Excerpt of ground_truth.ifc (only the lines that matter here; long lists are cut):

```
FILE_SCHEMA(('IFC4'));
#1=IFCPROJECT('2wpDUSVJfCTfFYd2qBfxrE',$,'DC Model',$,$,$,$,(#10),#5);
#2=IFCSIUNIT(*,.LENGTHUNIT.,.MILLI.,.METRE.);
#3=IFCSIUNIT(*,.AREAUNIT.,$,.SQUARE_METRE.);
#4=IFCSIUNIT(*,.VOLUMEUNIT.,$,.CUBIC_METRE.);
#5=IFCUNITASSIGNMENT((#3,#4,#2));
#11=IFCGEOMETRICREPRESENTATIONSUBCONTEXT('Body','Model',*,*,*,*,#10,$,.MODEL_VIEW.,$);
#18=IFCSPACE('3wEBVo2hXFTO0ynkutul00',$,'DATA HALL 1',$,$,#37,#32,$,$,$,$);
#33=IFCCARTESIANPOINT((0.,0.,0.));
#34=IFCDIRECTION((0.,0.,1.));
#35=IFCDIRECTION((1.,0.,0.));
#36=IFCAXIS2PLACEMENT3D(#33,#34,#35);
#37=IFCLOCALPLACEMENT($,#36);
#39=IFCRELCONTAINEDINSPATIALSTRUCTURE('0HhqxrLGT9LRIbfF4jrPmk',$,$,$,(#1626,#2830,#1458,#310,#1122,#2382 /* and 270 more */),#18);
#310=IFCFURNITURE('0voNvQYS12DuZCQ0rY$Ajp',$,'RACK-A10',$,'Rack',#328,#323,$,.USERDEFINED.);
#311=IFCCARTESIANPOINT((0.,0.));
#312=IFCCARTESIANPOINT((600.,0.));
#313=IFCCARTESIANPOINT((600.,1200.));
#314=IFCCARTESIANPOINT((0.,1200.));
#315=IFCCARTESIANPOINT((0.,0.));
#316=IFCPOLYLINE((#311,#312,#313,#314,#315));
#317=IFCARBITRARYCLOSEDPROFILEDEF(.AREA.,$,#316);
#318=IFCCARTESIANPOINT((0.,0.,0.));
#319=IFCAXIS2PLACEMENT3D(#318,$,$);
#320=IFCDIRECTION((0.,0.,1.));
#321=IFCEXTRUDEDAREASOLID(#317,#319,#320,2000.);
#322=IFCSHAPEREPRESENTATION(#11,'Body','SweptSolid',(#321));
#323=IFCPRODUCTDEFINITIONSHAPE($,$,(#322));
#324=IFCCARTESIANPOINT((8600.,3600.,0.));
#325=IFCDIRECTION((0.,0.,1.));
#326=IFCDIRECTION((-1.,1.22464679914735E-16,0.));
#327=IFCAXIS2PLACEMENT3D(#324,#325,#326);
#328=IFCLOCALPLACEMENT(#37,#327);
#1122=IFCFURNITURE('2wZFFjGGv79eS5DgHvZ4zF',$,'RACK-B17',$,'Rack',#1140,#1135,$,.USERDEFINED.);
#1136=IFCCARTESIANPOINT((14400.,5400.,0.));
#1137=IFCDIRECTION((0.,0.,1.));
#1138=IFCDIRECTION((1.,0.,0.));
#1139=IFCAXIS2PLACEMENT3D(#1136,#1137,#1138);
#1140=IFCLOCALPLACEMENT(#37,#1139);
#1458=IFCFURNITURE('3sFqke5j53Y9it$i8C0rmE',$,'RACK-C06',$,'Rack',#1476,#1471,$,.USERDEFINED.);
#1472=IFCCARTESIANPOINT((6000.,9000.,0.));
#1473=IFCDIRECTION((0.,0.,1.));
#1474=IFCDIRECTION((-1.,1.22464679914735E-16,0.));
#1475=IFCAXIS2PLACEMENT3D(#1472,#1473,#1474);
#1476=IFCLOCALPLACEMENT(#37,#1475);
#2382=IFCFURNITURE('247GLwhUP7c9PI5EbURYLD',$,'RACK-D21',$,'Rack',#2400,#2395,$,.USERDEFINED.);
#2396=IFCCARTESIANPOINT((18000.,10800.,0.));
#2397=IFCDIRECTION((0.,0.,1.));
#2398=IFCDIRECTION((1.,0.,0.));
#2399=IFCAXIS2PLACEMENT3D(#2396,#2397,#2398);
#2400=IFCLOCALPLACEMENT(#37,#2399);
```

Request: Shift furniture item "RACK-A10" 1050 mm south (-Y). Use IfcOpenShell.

```python
import ifcopenshell
import ifcopenshell.api.geometry
import ifcopenshell.util.placement
import ifcopenshell.util.unit

model = ifcopenshell.open("ground_truth.ifc")
unit_scale = ifcopenshell.util.unit.calculate_unit_scale(model)

item = model.by_guid("0voNvQYS12DuZCQ0rY$Ajp")
matrix = ifcopenshell.util.placement.get_local_placement(item.ObjectPlacement)
matrix[1, 3] -= 1.05 / unit_scale
ifcopenshell.api.geometry.edit_object_placement(model, product=item, matrix=matrix, is_si=False)

print(ifcopenshell.util.placement.get_local_placement(item.ObjectPlacement).round(3) + 0.0)

model.write("ground_truth_updated.ifc")
```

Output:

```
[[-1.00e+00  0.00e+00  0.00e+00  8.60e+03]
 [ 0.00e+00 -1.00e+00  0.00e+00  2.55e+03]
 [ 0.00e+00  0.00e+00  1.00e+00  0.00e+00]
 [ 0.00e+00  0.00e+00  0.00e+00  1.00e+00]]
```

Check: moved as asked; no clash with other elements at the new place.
